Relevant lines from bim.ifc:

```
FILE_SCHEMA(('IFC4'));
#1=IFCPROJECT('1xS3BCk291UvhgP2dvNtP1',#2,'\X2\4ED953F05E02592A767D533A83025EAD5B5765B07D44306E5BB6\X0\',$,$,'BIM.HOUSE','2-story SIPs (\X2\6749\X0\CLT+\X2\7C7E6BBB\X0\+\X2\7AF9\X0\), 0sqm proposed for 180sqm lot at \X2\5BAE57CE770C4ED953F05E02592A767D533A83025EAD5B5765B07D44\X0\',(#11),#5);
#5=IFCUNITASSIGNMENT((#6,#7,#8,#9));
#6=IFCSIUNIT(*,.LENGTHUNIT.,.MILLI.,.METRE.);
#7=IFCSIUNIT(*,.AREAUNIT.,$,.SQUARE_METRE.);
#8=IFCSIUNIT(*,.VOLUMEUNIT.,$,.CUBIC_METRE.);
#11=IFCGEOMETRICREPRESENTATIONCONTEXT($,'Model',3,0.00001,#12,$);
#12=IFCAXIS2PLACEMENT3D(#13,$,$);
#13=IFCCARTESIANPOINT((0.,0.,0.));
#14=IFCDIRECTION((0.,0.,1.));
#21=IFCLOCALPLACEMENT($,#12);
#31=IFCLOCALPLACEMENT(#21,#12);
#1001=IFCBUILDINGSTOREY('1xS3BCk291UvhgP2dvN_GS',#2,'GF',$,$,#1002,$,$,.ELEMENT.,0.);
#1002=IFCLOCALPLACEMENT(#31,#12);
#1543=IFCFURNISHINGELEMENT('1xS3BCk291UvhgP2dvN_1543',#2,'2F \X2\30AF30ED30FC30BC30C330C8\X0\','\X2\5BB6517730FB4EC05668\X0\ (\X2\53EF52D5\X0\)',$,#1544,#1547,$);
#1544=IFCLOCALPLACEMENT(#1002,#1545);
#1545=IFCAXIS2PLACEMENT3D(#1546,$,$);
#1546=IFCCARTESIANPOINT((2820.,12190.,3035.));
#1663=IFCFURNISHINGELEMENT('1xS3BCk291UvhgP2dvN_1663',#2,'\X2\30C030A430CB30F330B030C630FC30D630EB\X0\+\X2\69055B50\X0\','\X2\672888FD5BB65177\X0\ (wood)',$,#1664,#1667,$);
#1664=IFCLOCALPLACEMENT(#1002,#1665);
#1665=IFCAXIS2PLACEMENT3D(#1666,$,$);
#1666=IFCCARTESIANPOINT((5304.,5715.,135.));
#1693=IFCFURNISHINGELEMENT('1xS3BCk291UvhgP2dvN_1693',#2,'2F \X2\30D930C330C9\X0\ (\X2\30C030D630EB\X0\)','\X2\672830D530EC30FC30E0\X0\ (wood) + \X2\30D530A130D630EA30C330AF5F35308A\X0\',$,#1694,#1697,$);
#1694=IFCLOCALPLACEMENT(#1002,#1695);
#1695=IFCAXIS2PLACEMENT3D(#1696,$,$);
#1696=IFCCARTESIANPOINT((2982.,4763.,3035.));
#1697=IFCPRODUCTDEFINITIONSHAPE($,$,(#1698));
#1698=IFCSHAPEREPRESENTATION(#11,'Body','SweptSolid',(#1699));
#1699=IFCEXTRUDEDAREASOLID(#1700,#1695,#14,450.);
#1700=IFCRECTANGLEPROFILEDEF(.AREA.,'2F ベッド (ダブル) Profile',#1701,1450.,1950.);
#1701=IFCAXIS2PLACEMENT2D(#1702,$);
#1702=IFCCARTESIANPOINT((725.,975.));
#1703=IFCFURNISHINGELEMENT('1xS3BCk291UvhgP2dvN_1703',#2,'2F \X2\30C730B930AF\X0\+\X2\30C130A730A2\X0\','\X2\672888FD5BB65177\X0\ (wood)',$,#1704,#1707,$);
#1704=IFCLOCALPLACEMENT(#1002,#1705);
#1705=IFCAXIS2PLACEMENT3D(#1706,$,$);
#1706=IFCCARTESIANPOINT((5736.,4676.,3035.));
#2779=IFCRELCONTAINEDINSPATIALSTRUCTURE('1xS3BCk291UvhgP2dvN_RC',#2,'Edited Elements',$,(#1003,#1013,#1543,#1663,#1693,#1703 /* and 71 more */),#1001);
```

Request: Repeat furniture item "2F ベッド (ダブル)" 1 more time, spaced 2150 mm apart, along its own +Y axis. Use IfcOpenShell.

```python
import ifcopenshell
import ifcopenshell.api.geometry
import ifcopenshell.api.root
import ifcopenshell.util.element
import ifcopenshell.util.placement
import ifcopenshell.util.unit

model = ifcopenshell.open("bim.ifc")
unit_scale = ifcopenshell.util.unit.calculate_unit_scale(model)


def reuse_history(source, copy):
    """copy_class also copies each property set's owner history, people and application; keep the originals."""
    for rel in copy.IsDefinedBy:
        if rel.is_a("IfcRelDefinesByProperties") and (history := rel.RelatingPropertyDefinition.OwnerHistory):
            rel.RelatingPropertyDefinition.OwnerHistory = source.OwnerHistory
            ifcopenshell.util.element.remove_deep2(model, history)


source = model.by_id(1693)
base = ifcopenshell.util.placement.get_local_placement(source.ObjectPlacement)
step = base[:3, 1] * 2.15 / unit_scale

for i in range(1, 2):
    copy = ifcopenshell.api.root.copy_class(model, product=source)
    copy.Representation = ifcopenshell.util.element.copy_deep(
        model, source.Representation, exclude=["IfcGeometricRepresentationContext", "IfcRepresentationMap"]
    )
    reuse_history(source, copy)
    matrix = base.copy()
    matrix[:3, 3] += i * step
    print("added at", matrix[:3, 3].round(3) + 0.0)
    ifcopenshell.api.geometry.edit_object_placement(model, product=copy, matrix=matrix, is_si=False)

model.write("bim_rev.ifc")
```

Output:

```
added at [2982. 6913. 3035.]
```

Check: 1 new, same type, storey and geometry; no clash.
